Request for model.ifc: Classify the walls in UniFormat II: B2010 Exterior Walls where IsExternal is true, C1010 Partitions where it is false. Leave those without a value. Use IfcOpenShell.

First a look at what the model holds.

```python
import ifcopenshell
import ifcopenshell.util.element

model = ifcopenshell.open("model.ifc")
print(model.schema)
print("classifications:", [c.Name for c in model.by_type("IfcClassification")])
values = [ifcopenshell.util.element.get_pset(e, "Pset_WallCommon", "IsExternal") for e in model.by_type("IfcWall")]
for value in (True, False, None):
    print("IsExternal", value, values.count(value))
```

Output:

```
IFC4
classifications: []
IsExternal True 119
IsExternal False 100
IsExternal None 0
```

```python
import ifcopenshell
import ifcopenshell.api.classification
import ifcopenshell.util.element

model = ifcopenshell.open("model.ifc")

system = ifcopenshell.api.classification.add_classification(model, classification="UniFormat II")

walls = model.by_type("IfcWall")
external = {e: ifcopenshell.util.element.get_pset(e, "Pset_WallCommon", "IsExternal") for e in walls}
for flag, code, name in ((True, "B2010", "Exterior Walls"), (False, "C1010", "Partitions")):
    products = [e for e in walls if external[e] is flag]
    ifcopenshell.api.classification.add_reference(
        model, products=products, classification=system, identification=code, name=name
    )
    print(code, len(products))

model.write("model-out.ifc")
```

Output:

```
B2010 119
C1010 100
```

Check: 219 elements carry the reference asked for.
